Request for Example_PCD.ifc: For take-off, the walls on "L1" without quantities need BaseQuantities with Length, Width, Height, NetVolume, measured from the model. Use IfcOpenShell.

First a look at what the model holds.

```python
import ifcopenshell
import ifcopenshell.util.element
import ifcopenshell.util.unit

model = ifcopenshell.open("Example_PCD.ifc")
print(model.schema)
for unit_type in ("LENGTHUNIT", "AREAUNIT", "VOLUMEUNIT"):
    print(unit_type, ifcopenshell.util.unit.calculate_unit_scale(model, unit_type))
storey = next(s for s in model.by_type("IfcBuildingStorey") if s.Name == "L1")
walls = [e for e in ifcopenshell.util.element.get_decomposition(storey) if e.is_a("IfcWall")]
for e in sorted(walls, key=lambda e: e.id()):
    print(e.id(), e.is_a(), e.Name, list(ifcopenshell.util.element.get_psets(e, qtos_only=True)), sep=" | ")
```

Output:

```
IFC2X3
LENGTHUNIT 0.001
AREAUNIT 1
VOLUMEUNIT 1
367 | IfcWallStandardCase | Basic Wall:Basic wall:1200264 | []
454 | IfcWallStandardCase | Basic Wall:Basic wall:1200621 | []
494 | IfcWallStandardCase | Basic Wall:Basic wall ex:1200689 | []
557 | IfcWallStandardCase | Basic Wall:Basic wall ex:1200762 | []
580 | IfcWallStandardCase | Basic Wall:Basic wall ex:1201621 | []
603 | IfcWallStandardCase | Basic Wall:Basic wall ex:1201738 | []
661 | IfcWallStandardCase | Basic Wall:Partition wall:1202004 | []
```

```python
import ifcopenshell
import ifcopenshell.api.pset
import ifcopenshell.geom
import ifcopenshell.util.element
import ifcopenshell.util.shape
import ifcopenshell.util.unit

model = ifcopenshell.open("Example_PCD.ifc")
unit_scale = ifcopenshell.util.unit.calculate_unit_scale(model)
volume_scale = ifcopenshell.util.unit.calculate_unit_scale(model, "VOLUMEUNIT")
settings = ifcopenshell.geom.settings()

storey = next(s for s in model.by_type("IfcBuildingStorey") if s.Name == "L1")
walls = [e for e in ifcopenshell.util.element.get_decomposition(storey) if e.is_a("IfcWall")]

for e in sorted(walls, key=lambda e: e.id()):
    if ifcopenshell.util.element.get_psets(e, qtos_only=True, should_inherit=False):
        continue
    # Geometry comes back in metres, in the element's own axes.
    shape = ifcopenshell.geom.create_shape(settings, e)
    values = {
        "Length": ifcopenshell.util.shape.get_x(shape.geometry) / unit_scale,
        "Width": ifcopenshell.util.shape.get_y(shape.geometry) / unit_scale,
        "Height": ifcopenshell.util.shape.get_z(shape.geometry) / unit_scale,
        "NetVolume": ifcopenshell.util.shape.get_volume(shape.geometry) / volume_scale,
    }
    qto = ifcopenshell.api.pset.add_qto(model, product=e, name="BaseQuantities")
    ifcopenshell.api.pset.edit_qto(model, qto=qto, properties=values)
    print(e.id(), {k: round(v, 3) for k, v in values.items()})

model.write("Example_PCD_v2.ifc")
```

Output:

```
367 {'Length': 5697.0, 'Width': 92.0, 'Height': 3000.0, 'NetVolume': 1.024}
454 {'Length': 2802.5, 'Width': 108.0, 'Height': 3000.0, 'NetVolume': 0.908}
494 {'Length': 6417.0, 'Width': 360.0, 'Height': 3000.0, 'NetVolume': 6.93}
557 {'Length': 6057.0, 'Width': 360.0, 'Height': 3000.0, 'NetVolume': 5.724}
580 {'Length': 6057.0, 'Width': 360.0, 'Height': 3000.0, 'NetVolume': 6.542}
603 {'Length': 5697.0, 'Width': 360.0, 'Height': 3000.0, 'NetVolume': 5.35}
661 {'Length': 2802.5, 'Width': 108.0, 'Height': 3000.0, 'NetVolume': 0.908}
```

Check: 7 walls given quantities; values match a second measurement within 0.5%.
